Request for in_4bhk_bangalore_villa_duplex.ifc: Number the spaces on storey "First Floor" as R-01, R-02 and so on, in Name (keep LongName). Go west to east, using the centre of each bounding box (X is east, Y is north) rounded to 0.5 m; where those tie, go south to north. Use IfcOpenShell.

First a look at what the model holds.

```python
import ifcopenshell
import ifcopenshell.util.element
import ifcopenshell.util.placement

model = ifcopenshell.open("in_4bhk_bangalore_villa_duplex.ifc")
print(model.schema)
storey = next(s for s in model.by_type("IfcBuildingStorey") if s.Name == "First Floor")
spaces = [e for e in ifcopenshell.util.element.get_decomposition(storey) if e.is_a("IfcSpace")]
for e in sorted(spaces, key=lambda e: e.id()):
    origin = ifcopenshell.util.placement.get_local_placement(e.ObjectPlacement)[:3, 3]
    print(e.id(), e.Name, e.LongName, origin.round(2) + 0.0, sep=" | ")
```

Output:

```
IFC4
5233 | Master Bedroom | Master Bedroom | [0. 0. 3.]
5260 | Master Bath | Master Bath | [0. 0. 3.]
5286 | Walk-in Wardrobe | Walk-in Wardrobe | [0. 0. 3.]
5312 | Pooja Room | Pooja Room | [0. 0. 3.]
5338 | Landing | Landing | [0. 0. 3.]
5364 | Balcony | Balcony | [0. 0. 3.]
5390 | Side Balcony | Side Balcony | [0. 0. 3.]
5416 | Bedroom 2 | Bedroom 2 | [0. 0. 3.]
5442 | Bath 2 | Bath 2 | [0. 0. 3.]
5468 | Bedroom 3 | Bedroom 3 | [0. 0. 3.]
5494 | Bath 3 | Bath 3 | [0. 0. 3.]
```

```python
import ifcopenshell
import ifcopenshell.geom
import ifcopenshell.util.element
import ifcopenshell.util.shape

model = ifcopenshell.open("in_4bhk_bangalore_villa_duplex.ifc")
settings = ifcopenshell.geom.settings()
settings.set("use-world-coords", True)


def centre(element):
    shape = ifcopenshell.geom.create_shape(settings, element)
    return ifcopenshell.util.shape.get_bbox_centroid(shape.geometry)


storey = next(s for s in model.by_type("IfcBuildingStorey") if s.Name == "First Floor")
spaces = [e for e in ifcopenshell.util.element.get_decomposition(storey) if e.is_a("IfcSpace")]

# Insertion points can sit at a corner or the storey origin, so sort by the geometry (in metres).
centres = {e: centre(e) for e in spaces}
spaces.sort(key=lambda e: (round(centres[e][0] / 0.5), centres[e][1]))

for i, e in enumerate(spaces, start=1):
    number = f"R-{i:02d}"
    e.Name = number
    print(e.id(), number)

model.write("in_4bhk_bangalore_villa_duplex-out.ifc")
```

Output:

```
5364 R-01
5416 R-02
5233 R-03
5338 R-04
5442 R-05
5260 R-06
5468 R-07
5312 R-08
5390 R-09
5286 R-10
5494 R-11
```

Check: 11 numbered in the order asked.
